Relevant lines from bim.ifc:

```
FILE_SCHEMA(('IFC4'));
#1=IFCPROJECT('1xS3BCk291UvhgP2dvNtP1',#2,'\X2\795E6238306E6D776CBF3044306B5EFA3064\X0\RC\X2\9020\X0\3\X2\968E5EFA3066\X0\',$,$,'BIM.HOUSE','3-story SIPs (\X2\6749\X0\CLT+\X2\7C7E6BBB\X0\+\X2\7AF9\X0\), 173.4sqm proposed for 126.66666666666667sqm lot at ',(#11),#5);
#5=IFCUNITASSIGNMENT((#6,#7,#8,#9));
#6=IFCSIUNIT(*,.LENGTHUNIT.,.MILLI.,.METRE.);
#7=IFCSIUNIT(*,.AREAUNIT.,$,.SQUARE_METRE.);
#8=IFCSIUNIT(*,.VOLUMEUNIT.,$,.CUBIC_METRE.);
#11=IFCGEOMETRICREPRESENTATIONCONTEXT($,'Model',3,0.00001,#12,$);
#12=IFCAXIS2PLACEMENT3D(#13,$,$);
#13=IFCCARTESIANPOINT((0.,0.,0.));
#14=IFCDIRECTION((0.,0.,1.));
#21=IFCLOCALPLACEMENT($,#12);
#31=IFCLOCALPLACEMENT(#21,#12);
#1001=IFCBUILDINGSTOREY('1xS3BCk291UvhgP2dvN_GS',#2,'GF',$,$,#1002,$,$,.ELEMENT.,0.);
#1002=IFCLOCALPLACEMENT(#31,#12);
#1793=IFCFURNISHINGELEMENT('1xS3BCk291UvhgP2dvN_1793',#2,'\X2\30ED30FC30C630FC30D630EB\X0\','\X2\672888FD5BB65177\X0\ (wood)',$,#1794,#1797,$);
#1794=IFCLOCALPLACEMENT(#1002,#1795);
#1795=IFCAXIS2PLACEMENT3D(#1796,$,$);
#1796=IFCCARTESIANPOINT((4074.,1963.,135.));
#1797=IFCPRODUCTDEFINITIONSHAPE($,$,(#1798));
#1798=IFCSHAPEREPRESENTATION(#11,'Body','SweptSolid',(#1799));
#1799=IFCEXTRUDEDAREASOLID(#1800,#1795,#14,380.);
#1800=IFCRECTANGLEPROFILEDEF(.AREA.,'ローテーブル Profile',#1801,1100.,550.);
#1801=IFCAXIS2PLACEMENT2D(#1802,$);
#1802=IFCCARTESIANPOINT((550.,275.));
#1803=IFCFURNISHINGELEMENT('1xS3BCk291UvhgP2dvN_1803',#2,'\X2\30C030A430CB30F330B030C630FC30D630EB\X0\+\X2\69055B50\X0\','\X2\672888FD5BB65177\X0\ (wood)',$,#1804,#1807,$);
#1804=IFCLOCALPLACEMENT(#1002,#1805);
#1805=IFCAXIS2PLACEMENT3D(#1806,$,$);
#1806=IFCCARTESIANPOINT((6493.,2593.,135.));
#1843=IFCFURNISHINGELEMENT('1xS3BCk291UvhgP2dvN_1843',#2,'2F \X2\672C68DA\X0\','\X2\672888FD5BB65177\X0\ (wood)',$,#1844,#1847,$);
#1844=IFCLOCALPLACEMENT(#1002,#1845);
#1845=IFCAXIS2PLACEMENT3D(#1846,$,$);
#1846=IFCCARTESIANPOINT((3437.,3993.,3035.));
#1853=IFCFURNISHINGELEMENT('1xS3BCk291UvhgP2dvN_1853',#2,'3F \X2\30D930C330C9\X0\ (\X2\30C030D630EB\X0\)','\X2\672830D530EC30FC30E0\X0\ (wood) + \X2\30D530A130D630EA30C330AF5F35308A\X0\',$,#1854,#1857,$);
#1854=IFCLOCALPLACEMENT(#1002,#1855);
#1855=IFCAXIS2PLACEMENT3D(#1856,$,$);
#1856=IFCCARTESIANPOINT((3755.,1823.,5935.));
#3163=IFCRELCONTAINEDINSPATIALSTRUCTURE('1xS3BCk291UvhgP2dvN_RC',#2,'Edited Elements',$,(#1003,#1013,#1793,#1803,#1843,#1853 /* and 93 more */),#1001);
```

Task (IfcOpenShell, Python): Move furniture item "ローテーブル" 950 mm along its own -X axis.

```python
import ifcopenshell
import ifcopenshell.api.geometry
import ifcopenshell.util.placement
import ifcopenshell.util.unit

model = ifcopenshell.open("bim.ifc")
unit_scale = ifcopenshell.util.unit.calculate_unit_scale(model)

item = model.by_guid("1xS3BCk291UvhgP2dvN_1793")
matrix = ifcopenshell.util.placement.get_local_placement(item.ObjectPlacement)
matrix[:3, 3] -= matrix[:3, 0] * 0.95 / unit_scale
ifcopenshell.api.geometry.edit_object_placement(model, product=item, matrix=matrix, is_si=False)

print(ifcopenshell.util.placement.get_local_placement(item.ObjectPlacement).round(3) + 0.0)

model.write("bim-out.ifc")
```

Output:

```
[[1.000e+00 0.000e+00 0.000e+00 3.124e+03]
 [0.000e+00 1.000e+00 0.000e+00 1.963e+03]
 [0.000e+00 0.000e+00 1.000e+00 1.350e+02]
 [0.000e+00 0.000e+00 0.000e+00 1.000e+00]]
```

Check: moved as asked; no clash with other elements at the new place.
